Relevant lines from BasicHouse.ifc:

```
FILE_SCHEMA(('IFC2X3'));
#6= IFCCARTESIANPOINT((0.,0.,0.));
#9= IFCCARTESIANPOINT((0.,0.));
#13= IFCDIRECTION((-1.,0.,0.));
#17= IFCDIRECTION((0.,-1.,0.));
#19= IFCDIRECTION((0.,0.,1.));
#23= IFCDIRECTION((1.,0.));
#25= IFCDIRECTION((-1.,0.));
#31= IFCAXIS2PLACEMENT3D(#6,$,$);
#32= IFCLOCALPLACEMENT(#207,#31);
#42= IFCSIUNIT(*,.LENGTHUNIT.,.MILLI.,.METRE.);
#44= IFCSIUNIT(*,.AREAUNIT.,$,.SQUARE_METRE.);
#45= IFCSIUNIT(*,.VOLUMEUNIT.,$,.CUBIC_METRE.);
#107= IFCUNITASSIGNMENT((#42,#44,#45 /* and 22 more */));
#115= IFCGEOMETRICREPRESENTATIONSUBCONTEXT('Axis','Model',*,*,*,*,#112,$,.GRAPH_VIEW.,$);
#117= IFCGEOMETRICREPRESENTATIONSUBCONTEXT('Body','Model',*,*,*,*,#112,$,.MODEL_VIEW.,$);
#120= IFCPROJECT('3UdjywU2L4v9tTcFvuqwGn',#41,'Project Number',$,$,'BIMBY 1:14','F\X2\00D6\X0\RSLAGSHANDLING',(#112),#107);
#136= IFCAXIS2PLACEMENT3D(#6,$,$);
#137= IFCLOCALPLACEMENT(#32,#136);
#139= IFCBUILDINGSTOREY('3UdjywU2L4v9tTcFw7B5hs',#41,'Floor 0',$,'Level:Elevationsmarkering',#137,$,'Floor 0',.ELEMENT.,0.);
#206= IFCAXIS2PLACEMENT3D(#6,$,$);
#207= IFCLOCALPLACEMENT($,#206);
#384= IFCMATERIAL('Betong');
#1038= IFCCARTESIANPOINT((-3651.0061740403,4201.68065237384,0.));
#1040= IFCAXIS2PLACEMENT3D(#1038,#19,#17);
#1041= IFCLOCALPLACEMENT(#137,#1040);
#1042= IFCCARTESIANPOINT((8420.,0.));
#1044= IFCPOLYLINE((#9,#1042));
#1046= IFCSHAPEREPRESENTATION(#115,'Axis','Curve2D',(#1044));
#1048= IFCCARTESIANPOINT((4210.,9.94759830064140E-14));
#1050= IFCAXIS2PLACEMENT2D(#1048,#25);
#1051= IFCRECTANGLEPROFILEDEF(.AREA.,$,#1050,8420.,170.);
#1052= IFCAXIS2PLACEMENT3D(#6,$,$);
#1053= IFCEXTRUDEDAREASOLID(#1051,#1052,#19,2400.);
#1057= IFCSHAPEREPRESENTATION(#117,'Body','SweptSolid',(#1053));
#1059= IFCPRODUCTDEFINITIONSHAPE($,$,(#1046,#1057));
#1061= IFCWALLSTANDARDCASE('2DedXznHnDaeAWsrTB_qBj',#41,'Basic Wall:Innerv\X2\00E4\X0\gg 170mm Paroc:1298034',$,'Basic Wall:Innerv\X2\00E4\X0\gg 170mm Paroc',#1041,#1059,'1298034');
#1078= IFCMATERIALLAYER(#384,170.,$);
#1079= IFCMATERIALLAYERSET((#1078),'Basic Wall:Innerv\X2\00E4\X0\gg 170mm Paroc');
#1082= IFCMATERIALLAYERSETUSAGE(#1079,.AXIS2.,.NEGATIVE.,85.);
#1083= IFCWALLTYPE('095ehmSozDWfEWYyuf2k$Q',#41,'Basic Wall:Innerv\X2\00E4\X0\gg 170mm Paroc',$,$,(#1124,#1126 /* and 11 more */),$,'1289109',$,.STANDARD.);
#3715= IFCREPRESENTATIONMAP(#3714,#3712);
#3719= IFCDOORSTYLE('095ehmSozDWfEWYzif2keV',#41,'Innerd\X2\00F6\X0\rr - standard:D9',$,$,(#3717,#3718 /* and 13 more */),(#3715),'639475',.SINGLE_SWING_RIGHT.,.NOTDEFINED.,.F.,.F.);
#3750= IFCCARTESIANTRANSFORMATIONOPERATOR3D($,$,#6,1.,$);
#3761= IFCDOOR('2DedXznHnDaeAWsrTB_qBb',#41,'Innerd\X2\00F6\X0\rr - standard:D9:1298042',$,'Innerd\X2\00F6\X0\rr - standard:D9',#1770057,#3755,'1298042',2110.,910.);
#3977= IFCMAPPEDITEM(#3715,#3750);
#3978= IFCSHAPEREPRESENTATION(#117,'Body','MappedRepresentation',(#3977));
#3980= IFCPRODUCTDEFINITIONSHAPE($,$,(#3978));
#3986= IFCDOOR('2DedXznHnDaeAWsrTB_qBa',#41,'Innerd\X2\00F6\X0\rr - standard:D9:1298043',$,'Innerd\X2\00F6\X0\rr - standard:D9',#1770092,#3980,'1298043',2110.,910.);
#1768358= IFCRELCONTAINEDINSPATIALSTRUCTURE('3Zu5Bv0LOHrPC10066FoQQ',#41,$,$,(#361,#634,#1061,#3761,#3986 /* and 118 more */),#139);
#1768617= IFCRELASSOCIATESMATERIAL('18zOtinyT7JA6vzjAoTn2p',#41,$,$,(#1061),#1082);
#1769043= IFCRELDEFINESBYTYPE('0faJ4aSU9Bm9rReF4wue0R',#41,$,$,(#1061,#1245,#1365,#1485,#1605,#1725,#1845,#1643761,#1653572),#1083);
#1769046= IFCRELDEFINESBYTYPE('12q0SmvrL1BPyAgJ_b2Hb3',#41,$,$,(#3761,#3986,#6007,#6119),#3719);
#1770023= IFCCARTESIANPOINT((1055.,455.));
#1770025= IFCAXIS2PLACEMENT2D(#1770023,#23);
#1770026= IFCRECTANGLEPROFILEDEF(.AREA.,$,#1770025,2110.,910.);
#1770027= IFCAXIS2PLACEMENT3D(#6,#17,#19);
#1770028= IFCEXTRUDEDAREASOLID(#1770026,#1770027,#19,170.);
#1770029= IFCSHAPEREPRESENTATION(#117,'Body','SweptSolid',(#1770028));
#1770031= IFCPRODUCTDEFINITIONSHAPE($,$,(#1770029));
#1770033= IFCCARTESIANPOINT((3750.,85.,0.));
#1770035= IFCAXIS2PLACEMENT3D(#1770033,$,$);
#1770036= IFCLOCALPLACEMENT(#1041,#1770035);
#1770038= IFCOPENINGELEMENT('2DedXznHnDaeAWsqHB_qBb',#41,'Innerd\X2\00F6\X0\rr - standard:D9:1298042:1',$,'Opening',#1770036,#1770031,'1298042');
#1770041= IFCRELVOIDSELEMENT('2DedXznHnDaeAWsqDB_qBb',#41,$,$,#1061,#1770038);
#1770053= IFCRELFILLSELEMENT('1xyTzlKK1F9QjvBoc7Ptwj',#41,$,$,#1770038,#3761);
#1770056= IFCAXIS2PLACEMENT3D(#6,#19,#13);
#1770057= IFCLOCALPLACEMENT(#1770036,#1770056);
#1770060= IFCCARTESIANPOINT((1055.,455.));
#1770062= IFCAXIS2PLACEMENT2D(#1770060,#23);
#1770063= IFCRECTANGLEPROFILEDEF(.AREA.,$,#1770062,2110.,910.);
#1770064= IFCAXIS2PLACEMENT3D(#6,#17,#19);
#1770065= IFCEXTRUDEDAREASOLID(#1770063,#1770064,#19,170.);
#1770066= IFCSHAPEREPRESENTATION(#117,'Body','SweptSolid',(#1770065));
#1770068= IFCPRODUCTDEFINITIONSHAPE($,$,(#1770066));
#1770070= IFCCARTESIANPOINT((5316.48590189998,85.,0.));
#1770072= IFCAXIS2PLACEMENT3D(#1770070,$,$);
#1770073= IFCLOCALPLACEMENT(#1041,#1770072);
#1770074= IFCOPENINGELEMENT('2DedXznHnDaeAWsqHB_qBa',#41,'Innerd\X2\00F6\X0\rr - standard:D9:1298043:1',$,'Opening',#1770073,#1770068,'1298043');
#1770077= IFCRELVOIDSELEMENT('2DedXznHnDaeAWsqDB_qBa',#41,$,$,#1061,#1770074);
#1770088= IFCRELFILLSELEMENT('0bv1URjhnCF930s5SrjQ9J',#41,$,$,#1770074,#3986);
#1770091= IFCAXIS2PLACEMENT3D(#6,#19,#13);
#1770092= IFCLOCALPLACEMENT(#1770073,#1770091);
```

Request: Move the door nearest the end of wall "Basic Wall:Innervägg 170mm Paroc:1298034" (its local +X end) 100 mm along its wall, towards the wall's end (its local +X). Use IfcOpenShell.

```python
import ifcopenshell
import ifcopenshell.api.geometry
import ifcopenshell.util.placement

model = ifcopenshell.open("BasicHouse.ifc")

door = model.by_id(3986)
opening = door.FillsVoids[0].RelatingOpeningElement
wall = opening.VoidsElements[0].RelatingBuildingElement

wall_matrix = ifcopenshell.util.placement.get_local_placement(wall.ObjectPlacement)
shift = wall_matrix[:3, 0] * 100.0
before = ifcopenshell.util.placement.get_local_placement(door.ObjectPlacement)[:3, 3].copy()

# The door is placed relative to its opening, so it follows when the opening moves.
matrix = ifcopenshell.util.placement.get_local_placement(opening.ObjectPlacement)
matrix[:3, 3] += shift
ifcopenshell.api.geometry.edit_object_placement(
    model, product=opening, matrix=matrix, is_si=False, should_transform_children=True
)

after = ifcopenshell.util.placement.get_local_placement(door.ObjectPlacement)[:3, 3]
print("door moved by", (after - before).round(3) + 0.0)

model.write("BasicHouse-out.ifc")
```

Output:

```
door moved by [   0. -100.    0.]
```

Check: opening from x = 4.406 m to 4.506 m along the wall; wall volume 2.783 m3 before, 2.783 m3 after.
